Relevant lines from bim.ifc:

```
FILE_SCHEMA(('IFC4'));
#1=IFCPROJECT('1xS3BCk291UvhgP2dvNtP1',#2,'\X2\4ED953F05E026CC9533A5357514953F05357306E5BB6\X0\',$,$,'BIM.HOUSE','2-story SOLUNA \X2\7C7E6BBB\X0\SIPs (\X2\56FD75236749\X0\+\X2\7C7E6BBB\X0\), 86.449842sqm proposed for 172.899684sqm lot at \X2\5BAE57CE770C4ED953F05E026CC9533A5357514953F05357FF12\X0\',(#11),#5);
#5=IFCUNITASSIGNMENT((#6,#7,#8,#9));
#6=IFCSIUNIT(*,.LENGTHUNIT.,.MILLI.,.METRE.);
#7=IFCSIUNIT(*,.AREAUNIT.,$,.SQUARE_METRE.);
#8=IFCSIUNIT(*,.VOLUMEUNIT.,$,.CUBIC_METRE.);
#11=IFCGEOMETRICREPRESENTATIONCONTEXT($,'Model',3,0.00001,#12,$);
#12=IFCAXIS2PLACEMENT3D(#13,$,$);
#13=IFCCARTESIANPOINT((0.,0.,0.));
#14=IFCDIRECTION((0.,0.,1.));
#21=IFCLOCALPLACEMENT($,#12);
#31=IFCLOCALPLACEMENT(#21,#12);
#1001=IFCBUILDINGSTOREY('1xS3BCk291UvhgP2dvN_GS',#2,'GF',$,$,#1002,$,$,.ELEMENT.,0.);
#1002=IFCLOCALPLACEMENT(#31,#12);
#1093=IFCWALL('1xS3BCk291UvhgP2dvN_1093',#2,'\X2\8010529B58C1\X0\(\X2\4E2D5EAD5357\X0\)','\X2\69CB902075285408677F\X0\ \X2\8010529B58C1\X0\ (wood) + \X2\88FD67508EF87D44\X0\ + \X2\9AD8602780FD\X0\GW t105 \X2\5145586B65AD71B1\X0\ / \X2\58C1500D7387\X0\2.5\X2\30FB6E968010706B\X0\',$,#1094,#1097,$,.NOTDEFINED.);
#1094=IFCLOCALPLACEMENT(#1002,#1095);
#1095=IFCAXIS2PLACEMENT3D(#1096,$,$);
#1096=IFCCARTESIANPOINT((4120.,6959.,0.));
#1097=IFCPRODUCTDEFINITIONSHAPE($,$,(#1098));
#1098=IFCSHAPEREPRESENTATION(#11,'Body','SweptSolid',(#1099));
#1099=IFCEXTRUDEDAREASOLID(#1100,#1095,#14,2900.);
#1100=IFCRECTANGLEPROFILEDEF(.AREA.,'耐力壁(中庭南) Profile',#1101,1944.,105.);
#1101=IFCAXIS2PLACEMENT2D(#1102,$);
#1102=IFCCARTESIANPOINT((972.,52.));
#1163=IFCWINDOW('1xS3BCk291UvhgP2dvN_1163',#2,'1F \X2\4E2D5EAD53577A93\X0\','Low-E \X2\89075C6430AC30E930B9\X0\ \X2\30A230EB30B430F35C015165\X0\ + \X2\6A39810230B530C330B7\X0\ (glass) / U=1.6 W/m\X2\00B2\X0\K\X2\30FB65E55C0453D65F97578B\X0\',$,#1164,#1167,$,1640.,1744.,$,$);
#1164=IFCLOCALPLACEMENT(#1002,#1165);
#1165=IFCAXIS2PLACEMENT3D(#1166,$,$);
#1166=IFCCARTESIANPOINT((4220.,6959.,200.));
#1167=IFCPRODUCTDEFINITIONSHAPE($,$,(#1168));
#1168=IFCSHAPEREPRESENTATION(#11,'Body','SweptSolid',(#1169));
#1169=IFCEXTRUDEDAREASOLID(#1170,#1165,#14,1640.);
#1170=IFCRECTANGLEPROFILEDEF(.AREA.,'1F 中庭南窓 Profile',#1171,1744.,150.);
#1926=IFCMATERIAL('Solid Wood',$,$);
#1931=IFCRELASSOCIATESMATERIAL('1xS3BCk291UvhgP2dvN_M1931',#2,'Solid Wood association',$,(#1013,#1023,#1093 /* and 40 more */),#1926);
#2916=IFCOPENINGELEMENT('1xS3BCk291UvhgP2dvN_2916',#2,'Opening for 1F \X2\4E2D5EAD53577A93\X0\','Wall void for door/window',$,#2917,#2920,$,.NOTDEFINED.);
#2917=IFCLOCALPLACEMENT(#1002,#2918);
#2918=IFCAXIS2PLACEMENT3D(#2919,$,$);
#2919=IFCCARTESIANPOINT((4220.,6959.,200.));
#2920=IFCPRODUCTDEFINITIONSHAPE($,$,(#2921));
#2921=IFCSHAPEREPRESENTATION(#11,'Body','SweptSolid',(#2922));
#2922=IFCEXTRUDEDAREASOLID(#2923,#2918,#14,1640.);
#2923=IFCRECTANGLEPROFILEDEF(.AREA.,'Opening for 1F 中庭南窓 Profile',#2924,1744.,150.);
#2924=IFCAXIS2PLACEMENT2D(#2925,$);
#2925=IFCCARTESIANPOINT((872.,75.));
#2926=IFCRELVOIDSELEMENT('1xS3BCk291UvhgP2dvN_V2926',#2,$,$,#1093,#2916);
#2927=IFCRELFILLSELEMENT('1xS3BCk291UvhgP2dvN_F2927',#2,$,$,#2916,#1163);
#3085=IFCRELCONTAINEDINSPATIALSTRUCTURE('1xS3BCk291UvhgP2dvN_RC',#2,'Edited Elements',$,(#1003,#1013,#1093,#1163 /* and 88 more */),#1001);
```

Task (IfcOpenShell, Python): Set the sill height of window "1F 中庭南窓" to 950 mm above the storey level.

```python
import numpy as np
import ifcopenshell
import ifcopenshell.api.geometry
import ifcopenshell.geom
import ifcopenshell.util.element
import ifcopenshell.util.placement
import ifcopenshell.util.shape
import ifcopenshell.util.unit

model = ifcopenshell.open("bim.ifc")
unit_scale = ifcopenshell.util.unit.calculate_unit_scale(model)

window = model.by_id(1163)
opening = window.FillsVoids[0].RelatingOpeningElement
storey = ifcopenshell.util.element.get_container(window, ifc_class="IfcBuildingStorey")
level = ifcopenshell.util.placement.get_local_placement(storey.ObjectPlacement)[2, 3]

# The opening's origin need not be at the sill, so measure its lowest point.
shape = ifcopenshell.geom.create_shape(ifcopenshell.geom.settings(), opening)
bottom = ifcopenshell.util.shape.get_shape_bottom_elevation(shape, shape.geometry) / unit_scale
dz = level + 950.0 - bottom

shift = np.array([0.0, 0.0, dz])
# The window is not placed relative to its opening, so move both.
for product in (opening, window):
    matrix = ifcopenshell.util.placement.get_local_placement(product.ObjectPlacement)
    matrix[:3, 3] += shift
    ifcopenshell.api.geometry.edit_object_placement(model, product=product, matrix=matrix, is_si=False)

print(f"moved by {dz * unit_scale:+.3f} m")

model.write("bim_updated.ifc")
```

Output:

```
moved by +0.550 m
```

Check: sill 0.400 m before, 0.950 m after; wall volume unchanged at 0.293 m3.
